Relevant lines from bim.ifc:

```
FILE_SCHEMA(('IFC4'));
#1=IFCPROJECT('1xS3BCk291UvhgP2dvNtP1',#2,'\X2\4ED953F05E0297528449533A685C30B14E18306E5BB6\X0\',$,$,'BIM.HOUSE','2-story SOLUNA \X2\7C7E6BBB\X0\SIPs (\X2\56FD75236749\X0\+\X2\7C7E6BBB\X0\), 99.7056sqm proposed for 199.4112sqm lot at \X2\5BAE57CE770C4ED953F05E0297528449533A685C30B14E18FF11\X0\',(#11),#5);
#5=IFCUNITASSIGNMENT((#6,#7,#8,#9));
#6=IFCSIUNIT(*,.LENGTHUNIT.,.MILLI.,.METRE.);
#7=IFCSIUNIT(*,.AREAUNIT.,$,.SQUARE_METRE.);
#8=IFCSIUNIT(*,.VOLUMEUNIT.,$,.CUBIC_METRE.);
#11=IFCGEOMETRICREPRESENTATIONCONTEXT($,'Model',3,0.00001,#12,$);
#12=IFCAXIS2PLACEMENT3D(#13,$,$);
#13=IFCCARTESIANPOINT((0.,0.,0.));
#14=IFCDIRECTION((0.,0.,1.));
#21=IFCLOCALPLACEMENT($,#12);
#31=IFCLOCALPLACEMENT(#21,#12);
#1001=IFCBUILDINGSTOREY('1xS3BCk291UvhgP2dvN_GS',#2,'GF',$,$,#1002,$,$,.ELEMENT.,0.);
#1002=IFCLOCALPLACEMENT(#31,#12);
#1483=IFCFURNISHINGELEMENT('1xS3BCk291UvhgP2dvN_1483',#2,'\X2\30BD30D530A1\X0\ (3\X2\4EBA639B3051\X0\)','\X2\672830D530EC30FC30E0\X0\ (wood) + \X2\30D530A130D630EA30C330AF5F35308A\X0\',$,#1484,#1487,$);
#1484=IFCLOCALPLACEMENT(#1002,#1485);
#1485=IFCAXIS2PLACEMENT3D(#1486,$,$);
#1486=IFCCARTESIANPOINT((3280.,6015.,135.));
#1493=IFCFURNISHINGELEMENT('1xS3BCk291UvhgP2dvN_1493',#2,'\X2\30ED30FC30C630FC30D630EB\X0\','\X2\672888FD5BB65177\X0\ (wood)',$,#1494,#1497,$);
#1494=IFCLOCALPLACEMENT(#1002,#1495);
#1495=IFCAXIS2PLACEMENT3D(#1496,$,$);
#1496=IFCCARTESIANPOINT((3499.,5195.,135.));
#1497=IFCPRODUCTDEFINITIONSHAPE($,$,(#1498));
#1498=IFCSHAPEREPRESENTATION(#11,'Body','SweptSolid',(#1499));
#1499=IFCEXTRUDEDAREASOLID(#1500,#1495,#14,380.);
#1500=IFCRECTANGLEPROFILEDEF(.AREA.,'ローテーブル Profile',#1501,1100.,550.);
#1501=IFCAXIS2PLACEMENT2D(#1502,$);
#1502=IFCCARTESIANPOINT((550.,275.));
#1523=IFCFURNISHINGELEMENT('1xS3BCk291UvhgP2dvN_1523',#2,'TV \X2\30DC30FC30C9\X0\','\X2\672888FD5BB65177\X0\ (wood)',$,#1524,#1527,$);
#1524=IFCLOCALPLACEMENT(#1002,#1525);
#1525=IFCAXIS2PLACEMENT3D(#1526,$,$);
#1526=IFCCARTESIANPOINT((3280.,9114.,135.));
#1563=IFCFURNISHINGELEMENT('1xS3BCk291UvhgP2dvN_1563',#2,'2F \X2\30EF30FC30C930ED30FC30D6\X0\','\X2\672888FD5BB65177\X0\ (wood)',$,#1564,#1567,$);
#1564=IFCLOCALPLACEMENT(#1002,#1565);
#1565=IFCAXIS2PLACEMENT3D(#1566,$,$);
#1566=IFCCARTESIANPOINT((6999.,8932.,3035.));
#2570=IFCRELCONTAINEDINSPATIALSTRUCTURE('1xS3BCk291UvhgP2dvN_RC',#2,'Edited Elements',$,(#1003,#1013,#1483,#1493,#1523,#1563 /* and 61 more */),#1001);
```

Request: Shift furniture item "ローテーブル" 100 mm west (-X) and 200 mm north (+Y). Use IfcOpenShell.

```python
import ifcopenshell
import ifcopenshell.api.geometry
import ifcopenshell.util.placement

model = ifcopenshell.open("bim.ifc")

item = model.by_guid("1xS3BCk291UvhgP2dvN_1493")
matrix = ifcopenshell.util.placement.get_local_placement(item.ObjectPlacement)
matrix[0, 3] -= 100.0
matrix[1, 3] += 200.0
ifcopenshell.api.geometry.edit_object_placement(model, product=item, matrix=matrix, is_si=False)

print(ifcopenshell.util.placement.get_local_placement(item.ObjectPlacement).round(3) + 0.0)

model.write("bim-out.ifc")
```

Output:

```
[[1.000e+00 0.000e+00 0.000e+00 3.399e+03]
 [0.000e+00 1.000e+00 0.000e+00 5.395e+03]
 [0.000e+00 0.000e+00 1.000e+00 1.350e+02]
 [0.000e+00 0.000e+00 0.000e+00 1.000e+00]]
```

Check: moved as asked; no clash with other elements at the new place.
